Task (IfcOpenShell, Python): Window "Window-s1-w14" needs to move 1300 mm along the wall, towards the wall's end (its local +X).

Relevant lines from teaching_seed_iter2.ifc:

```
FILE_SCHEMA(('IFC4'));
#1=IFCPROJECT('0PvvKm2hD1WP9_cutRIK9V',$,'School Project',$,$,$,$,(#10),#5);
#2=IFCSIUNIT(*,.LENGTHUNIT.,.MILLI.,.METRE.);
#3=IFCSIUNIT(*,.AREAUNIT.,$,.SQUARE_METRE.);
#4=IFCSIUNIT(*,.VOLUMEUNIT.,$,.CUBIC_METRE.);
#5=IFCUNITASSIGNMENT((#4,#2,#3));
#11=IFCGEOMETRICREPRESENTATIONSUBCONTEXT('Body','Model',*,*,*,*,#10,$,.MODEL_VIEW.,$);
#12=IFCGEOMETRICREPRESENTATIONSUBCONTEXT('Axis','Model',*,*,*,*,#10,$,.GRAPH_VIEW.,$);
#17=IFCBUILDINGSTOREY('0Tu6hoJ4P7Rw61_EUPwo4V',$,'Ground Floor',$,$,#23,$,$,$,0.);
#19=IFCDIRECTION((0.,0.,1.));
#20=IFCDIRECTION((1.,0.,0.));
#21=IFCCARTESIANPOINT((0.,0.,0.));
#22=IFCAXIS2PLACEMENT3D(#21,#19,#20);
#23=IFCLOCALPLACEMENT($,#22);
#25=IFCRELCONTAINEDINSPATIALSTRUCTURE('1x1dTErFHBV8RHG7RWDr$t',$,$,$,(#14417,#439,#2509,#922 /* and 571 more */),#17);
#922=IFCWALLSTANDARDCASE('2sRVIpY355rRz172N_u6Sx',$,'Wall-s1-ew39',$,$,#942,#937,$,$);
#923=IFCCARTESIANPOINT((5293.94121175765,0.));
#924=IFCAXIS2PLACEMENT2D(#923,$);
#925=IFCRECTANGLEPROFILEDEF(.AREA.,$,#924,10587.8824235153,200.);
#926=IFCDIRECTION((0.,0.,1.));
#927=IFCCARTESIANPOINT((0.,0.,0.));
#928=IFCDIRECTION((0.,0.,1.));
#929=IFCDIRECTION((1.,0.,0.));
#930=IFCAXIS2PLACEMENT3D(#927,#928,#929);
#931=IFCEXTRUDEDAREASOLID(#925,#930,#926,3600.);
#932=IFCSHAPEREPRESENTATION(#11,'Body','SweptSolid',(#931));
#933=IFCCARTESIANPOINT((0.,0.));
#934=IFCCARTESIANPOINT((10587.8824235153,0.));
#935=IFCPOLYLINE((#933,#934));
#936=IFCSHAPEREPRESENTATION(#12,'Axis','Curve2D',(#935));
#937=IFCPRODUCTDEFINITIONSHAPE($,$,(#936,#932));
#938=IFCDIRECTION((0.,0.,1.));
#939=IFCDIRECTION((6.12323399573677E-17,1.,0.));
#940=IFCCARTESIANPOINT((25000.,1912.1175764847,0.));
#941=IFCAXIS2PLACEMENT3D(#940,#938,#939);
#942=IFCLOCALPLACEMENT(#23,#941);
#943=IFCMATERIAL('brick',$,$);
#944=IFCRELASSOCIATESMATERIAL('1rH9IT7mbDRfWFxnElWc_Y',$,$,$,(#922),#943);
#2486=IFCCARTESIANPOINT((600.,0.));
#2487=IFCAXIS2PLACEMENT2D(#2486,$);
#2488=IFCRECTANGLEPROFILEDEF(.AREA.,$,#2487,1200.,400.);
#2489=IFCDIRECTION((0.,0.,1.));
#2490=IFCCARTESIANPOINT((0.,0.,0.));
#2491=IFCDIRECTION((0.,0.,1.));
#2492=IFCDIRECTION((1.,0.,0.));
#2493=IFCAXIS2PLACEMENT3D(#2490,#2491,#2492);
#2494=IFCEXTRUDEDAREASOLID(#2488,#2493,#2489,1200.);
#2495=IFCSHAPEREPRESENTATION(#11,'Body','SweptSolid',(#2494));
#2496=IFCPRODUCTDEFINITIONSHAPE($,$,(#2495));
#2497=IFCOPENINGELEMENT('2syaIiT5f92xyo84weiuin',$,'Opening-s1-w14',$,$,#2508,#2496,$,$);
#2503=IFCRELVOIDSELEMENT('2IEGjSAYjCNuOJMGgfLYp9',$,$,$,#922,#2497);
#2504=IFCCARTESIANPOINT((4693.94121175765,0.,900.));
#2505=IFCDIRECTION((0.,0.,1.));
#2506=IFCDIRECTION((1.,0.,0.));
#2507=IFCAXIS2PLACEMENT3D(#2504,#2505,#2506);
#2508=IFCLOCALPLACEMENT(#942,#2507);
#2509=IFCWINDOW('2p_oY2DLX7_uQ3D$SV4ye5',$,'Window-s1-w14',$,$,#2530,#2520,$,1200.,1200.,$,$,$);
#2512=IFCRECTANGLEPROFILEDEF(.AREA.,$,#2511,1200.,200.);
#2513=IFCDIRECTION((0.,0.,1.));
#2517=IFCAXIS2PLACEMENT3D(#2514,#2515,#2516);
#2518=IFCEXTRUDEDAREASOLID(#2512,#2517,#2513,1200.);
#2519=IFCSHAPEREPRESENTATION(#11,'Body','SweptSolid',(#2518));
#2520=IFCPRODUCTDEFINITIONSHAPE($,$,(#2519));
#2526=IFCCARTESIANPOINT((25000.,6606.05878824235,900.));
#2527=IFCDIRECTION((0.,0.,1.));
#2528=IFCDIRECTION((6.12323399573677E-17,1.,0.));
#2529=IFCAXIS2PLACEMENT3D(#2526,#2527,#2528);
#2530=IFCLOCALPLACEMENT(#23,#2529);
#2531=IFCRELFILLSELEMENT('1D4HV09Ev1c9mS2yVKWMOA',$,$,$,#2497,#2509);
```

```python
import ifcopenshell
import ifcopenshell.api.geometry
import ifcopenshell.util.placement
import ifcopenshell.util.unit

model = ifcopenshell.open("teaching_seed_iter2.ifc")
unit_scale = ifcopenshell.util.unit.calculate_unit_scale(model)

window = model.by_guid("2p_oY2DLX7_uQ3D$SV4ye5")
opening = window.FillsVoids[0].RelatingOpeningElement
wall = opening.VoidsElements[0].RelatingBuildingElement

wall_matrix = ifcopenshell.util.placement.get_local_placement(wall.ObjectPlacement)
shift = wall_matrix[:3, 0] * 1.3 / unit_scale
before = ifcopenshell.util.placement.get_local_placement(window.ObjectPlacement)[:3, 3].copy()

# The window is not placed relative to its opening, so move both.
for product in (opening, window):
    matrix = ifcopenshell.util.placement.get_local_placement(product.ObjectPlacement)
    matrix[:3, 3] += shift
    ifcopenshell.api.geometry.edit_object_placement(model, product=product, matrix=matrix, is_si=False)

after = ifcopenshell.util.placement.get_local_placement(window.ObjectPlacement)[:3, 3]
print("window moved by", (after - before).round(3) + 0.0)

model.write("teaching_seed_iter2_edited.ifc")
```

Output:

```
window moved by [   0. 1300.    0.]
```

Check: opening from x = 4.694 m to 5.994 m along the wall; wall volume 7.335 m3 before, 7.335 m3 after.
